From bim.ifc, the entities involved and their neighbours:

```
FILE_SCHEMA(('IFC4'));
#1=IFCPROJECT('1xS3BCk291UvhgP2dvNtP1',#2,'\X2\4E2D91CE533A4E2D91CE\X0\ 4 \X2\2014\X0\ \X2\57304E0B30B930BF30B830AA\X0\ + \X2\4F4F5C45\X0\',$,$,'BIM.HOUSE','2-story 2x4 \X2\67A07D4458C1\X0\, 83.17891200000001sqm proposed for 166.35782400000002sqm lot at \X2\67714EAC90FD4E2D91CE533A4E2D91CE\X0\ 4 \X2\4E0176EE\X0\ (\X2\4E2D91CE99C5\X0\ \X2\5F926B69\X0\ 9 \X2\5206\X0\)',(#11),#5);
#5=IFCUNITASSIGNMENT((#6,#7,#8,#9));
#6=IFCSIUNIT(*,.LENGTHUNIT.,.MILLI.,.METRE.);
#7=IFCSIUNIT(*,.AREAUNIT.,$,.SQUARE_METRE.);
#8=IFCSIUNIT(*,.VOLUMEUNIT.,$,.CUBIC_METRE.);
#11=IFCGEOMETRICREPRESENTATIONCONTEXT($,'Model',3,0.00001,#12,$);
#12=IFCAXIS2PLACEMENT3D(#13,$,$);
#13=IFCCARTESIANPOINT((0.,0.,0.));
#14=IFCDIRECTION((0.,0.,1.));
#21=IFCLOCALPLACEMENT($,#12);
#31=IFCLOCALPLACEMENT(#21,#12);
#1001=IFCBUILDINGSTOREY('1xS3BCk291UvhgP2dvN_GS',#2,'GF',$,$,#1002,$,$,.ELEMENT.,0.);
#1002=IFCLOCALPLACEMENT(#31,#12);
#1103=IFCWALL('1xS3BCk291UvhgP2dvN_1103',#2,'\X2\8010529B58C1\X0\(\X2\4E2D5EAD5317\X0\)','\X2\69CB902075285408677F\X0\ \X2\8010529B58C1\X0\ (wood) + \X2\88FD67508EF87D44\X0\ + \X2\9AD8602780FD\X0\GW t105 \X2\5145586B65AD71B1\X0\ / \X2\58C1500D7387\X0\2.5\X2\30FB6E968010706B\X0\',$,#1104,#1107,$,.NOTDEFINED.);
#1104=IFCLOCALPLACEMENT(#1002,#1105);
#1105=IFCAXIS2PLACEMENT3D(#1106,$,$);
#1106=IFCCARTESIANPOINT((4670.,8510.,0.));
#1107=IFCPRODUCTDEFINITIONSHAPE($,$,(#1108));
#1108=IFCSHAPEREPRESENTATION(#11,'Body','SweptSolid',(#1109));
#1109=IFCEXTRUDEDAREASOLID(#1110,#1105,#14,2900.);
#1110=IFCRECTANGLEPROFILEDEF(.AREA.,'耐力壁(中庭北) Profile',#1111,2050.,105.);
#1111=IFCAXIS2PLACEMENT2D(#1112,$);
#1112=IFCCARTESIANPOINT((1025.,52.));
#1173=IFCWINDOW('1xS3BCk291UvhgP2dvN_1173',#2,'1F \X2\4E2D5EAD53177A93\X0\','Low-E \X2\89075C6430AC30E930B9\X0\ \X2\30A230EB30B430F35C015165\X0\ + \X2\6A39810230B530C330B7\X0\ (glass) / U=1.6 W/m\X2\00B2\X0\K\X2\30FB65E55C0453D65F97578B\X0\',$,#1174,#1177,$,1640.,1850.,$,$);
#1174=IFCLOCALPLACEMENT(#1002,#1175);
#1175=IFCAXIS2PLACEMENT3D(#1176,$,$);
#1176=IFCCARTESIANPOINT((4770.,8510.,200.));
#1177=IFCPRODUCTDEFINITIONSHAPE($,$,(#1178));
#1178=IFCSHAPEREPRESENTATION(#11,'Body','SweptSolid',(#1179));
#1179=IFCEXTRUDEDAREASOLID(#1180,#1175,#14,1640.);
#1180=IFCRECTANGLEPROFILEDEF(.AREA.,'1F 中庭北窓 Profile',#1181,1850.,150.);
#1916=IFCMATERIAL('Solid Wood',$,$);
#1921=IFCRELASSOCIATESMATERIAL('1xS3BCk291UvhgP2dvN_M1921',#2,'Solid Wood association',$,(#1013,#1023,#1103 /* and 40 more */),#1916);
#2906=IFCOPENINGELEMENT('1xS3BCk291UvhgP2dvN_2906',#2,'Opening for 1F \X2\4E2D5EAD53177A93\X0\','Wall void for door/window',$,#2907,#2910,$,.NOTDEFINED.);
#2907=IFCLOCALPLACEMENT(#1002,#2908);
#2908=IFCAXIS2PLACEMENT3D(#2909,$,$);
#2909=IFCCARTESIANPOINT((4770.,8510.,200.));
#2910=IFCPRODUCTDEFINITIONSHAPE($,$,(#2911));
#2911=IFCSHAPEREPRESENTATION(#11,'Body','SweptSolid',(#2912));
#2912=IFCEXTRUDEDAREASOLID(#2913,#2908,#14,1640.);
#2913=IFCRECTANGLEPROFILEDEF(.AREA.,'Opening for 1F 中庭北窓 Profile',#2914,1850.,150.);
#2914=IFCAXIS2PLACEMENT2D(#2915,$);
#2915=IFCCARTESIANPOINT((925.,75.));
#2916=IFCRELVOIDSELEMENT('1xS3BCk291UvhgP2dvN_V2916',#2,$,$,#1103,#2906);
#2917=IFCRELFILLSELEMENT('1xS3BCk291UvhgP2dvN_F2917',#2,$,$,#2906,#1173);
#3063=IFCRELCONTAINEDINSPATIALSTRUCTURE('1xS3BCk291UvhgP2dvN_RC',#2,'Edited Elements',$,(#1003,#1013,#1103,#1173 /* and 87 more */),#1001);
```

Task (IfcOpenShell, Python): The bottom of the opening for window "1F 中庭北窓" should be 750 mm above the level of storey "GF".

```python
import numpy as np
import ifcopenshell
import ifcopenshell.api.geometry
import ifcopenshell.geom
import ifcopenshell.util.element
import ifcopenshell.util.placement
import ifcopenshell.util.shape
import ifcopenshell.util.unit

model = ifcopenshell.open("bim.ifc")
unit_scale = ifcopenshell.util.unit.calculate_unit_scale(model)

window = model.by_guid("1xS3BCk291UvhgP2dvN_1173")
opening = window.FillsVoids[0].RelatingOpeningElement
storey = ifcopenshell.util.element.get_container(window, ifc_class="IfcBuildingStorey")
level = ifcopenshell.util.placement.get_local_placement(storey.ObjectPlacement)[2, 3]

# The opening's origin need not be at the sill, so measure its lowest point.
shape = ifcopenshell.geom.create_shape(ifcopenshell.geom.settings(), opening)
bottom = ifcopenshell.util.shape.get_shape_bottom_elevation(shape, shape.geometry) / unit_scale
dz = level + 0.75 / unit_scale - bottom

shift = np.array([0.0, 0.0, dz])
# The window is not placed relative to its opening, so move both.
for product in (opening, window):
    matrix = ifcopenshell.util.placement.get_local_placement(product.ObjectPlacement)
    matrix[:3, 3] += shift
    ifcopenshell.api.geometry.edit_object_placement(model, product=product, matrix=matrix, is_si=False)

print(f"moved by {dz * unit_scale:+.3f} m")

model.write("bim-out.ifc")
```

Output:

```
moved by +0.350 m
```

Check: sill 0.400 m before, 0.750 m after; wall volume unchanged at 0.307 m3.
